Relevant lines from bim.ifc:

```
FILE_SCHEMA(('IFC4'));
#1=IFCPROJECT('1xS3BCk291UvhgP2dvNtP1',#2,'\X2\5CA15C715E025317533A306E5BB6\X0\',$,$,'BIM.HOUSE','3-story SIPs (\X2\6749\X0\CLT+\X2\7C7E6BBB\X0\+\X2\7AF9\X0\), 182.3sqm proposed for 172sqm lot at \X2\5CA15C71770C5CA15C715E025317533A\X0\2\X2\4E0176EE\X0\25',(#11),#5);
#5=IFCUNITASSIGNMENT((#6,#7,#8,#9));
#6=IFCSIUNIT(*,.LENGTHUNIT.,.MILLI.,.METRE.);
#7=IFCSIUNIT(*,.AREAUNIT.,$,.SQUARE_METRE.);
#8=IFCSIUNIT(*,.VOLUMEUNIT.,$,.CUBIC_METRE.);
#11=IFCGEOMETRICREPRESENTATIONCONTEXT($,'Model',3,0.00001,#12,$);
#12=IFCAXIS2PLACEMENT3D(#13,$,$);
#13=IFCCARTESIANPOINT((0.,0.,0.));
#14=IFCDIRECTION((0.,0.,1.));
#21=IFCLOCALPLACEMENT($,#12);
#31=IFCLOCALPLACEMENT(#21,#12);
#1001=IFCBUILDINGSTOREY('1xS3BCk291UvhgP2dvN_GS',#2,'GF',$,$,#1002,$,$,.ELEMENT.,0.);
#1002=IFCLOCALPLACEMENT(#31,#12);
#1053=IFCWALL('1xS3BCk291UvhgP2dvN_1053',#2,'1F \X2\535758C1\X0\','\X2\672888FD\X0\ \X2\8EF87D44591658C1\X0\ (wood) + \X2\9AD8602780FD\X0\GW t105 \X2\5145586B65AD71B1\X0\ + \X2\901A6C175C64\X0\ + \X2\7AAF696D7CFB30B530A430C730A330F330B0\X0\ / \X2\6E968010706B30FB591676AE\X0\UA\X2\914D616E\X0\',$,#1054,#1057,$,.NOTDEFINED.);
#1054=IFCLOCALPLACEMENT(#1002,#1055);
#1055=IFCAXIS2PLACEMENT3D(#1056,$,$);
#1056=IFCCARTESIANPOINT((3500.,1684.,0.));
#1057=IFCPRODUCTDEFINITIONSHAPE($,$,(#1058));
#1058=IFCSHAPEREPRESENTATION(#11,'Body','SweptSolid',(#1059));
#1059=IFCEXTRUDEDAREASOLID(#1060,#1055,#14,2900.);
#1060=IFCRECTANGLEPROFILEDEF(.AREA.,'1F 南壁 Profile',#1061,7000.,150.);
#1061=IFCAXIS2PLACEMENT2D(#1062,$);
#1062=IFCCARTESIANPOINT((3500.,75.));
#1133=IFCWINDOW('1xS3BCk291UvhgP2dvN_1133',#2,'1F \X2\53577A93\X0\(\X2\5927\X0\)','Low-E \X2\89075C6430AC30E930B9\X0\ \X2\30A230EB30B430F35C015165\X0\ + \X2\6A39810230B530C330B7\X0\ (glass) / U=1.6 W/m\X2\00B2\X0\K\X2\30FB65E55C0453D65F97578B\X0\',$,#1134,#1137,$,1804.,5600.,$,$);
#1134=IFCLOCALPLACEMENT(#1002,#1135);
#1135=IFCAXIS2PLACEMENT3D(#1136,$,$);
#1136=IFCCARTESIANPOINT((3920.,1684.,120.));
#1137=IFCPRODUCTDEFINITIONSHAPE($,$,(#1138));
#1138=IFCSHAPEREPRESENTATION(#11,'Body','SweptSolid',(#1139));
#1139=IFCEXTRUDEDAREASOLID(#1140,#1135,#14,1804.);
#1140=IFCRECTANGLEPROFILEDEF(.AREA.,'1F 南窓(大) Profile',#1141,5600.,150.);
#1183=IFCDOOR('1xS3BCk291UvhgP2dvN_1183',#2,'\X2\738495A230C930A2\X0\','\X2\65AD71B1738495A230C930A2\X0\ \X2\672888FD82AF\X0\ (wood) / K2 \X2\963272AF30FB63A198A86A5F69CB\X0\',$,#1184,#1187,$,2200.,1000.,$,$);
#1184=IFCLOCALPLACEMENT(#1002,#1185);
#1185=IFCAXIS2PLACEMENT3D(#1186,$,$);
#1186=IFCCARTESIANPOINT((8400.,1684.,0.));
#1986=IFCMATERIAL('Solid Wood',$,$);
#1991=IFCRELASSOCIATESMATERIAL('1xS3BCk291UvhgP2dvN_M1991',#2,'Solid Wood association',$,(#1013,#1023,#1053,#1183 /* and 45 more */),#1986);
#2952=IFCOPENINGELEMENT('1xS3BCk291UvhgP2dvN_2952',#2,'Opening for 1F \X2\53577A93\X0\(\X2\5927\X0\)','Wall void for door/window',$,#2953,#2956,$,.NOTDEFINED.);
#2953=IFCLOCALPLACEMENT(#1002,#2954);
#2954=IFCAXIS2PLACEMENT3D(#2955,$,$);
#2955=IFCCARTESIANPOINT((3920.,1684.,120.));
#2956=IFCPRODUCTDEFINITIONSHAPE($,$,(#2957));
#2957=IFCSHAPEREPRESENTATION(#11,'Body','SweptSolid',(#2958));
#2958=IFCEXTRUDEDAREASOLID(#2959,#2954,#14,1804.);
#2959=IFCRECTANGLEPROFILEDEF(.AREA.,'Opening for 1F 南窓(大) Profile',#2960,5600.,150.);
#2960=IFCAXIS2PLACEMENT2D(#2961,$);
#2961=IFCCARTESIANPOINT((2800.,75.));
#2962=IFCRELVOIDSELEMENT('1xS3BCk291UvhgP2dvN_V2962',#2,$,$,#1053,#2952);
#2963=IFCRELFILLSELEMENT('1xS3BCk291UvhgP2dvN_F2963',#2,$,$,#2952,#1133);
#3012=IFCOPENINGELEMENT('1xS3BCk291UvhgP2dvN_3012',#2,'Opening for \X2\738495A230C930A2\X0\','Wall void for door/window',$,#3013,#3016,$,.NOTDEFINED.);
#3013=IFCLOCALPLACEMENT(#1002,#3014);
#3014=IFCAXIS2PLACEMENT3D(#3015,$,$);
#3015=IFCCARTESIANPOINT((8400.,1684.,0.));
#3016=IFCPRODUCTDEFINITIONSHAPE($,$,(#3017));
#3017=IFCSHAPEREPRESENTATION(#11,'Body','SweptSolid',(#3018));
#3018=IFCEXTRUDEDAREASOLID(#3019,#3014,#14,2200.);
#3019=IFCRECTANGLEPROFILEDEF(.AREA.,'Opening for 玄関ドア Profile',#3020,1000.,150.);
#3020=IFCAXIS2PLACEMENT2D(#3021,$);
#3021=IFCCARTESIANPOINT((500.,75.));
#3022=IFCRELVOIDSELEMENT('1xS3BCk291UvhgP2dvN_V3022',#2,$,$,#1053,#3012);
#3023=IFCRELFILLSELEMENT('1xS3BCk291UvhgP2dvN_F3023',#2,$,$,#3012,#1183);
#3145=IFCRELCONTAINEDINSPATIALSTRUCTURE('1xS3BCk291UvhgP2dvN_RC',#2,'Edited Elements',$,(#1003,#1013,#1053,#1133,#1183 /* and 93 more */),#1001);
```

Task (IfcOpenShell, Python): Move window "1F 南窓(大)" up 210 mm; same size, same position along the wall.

```python
import numpy as np
import ifcopenshell
import ifcopenshell.api.geometry
import ifcopenshell.util.placement
import ifcopenshell.util.unit

model = ifcopenshell.open("bim.ifc")
unit_scale = ifcopenshell.util.unit.calculate_unit_scale(model)

window = model.by_guid("1xS3BCk291UvhgP2dvN_1133")
opening = window.FillsVoids[0].RelatingOpeningElement
dz = 0.21 / unit_scale

shift = np.array([0.0, 0.0, dz])
# The window is not placed relative to its opening, so move both.
for product in (opening, window):
    matrix = ifcopenshell.util.placement.get_local_placement(product.ObjectPlacement)
    matrix[:3, 3] += shift
    ifcopenshell.api.geometry.edit_object_placement(model, product=product, matrix=matrix, is_si=False)

print(f"moved by {dz * unit_scale:+.3f} m")

model.write("bim_updated.ifc")
```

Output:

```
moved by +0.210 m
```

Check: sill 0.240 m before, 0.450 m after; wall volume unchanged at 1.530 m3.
